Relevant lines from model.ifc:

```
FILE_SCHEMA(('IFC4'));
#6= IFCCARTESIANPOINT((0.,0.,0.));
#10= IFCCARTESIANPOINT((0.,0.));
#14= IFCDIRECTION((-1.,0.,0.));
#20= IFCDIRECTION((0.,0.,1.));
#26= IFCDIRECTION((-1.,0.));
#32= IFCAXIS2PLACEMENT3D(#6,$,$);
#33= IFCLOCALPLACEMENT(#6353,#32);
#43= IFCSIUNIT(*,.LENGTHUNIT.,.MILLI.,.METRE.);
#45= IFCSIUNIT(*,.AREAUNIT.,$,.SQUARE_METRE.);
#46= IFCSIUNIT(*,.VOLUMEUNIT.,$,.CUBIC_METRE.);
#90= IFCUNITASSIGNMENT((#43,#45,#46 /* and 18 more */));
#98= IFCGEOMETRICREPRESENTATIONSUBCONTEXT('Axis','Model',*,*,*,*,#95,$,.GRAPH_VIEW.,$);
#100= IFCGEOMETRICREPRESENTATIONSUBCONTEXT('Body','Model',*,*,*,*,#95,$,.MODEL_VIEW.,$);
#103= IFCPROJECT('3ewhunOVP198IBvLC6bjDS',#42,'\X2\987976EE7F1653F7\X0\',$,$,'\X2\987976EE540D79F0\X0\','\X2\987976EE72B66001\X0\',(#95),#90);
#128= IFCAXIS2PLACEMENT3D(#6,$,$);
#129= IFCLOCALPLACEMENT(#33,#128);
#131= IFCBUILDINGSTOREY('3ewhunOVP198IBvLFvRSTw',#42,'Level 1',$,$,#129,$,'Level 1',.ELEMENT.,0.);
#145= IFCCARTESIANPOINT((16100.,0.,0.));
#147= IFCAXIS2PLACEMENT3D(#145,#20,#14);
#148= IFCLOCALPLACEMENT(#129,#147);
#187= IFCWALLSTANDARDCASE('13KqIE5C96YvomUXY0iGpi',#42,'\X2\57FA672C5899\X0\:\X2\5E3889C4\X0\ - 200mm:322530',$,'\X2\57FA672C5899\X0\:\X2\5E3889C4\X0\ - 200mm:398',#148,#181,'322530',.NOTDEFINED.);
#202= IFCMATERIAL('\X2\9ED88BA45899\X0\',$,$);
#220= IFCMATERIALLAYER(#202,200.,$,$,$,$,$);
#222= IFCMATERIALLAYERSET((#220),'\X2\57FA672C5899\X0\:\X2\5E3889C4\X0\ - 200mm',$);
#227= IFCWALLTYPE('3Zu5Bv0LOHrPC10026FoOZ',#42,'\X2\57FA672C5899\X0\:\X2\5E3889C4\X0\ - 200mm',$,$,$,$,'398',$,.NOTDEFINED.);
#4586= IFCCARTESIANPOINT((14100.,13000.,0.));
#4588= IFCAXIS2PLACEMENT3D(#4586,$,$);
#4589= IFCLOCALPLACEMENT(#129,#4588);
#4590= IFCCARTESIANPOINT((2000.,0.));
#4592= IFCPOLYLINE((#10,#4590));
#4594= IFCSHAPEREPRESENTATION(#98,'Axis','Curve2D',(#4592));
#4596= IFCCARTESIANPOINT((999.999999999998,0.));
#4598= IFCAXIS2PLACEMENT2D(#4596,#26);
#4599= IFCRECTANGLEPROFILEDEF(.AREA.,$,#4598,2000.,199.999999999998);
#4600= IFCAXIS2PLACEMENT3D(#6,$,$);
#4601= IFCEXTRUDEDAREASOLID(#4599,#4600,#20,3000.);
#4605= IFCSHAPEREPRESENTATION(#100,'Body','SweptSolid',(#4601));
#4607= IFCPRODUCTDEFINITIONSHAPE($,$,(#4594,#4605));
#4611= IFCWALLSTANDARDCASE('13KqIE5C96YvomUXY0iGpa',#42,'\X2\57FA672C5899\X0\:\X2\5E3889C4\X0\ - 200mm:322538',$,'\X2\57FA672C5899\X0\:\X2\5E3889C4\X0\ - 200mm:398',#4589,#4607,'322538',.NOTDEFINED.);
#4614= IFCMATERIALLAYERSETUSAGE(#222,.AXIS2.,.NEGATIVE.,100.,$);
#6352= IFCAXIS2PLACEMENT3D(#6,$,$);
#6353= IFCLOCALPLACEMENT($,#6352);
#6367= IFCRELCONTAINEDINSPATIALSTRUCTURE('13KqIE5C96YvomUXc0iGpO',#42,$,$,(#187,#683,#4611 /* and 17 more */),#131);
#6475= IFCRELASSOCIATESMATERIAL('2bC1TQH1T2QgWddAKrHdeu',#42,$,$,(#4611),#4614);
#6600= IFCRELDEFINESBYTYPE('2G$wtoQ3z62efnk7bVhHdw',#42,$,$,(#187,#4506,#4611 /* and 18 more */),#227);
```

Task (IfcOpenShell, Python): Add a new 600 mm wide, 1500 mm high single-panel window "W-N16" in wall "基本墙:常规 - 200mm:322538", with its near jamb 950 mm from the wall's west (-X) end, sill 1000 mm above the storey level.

```python
import numpy as np
import ifcopenshell
import ifcopenshell.api.feature
import ifcopenshell.api.geometry
import ifcopenshell.api.root
import ifcopenshell.api.spatial
import ifcopenshell.geom
import ifcopenshell.util.element
import ifcopenshell.util.placement
import ifcopenshell.util.representation
import ifcopenshell.util.shape
import ifcopenshell.util.unit

model = ifcopenshell.open("model.ifc")
unit_scale = ifcopenshell.util.unit.calculate_unit_scale(model)
settings = ifcopenshell.geom.settings()


def volume(element):
    """Net volume in cubic metres, openings subtracted."""
    shape = ifcopenshell.geom.create_shape(settings, element)
    return ifcopenshell.util.shape.get_volume(shape.geometry)


wall = model.by_guid("13KqIE5C96YvomUXY0iGpa")
storey = ifcopenshell.util.element.get_container(wall, ifc_class="IfcBuildingStorey")
context = ifcopenshell.util.representation.get_context(model, "Model", "Body", "MODEL_VIEW")
before = volume(wall)

width, height, from_end, sill = 0.6, 1.5, 0.95, 1  # metres

# The wall runs along its own X axis, and the end named is its -X end.
wall_shape = ifcopenshell.geom.create_shape(settings, wall)
x, y, z = ifcopenshell.util.shape.get_vertices(wall_shape.geometry).T
start = x.min() + from_end
face, thickness = float(y.min()), float(y.max() - y.min())
wall_matrix = ifcopenshell.util.placement.get_local_placement(wall.ObjectPlacement)
level = ifcopenshell.util.placement.get_local_placement(storey.ObjectPlacement)[2, 3]


def in_wall(x, y):
    """Placement at x, y metres in the wall's axes, at sill height."""
    matrix = wall_matrix.copy()
    matrix[:, 3] = wall_matrix @ np.array([x / unit_scale, y / unit_scale, 0.0, 1.0])
    matrix[2, 3] = level + sill / unit_scale
    return matrix


# Opening: a box that overshoots both wall faces by 50 mm.
opening = ifcopenshell.api.root.create_entity(model, ifc_class="IfcOpeningElement", predefined_type="OPENING")
box = ifcopenshell.api.geometry.add_wall_representation(
    model, context=context, length=width, height=height, thickness=thickness + 0.1
)
ifcopenshell.api.geometry.assign_representation(model, product=opening, representation=box)
ifcopenshell.api.geometry.edit_object_placement(model, product=opening, matrix=in_wall(start, face - 0.05), is_si=False)
ifcopenshell.api.feature.add_feature(model, feature=opening, element=wall)

window = ifcopenshell.api.root.create_entity(model, ifc_class="IfcWindow", name="W-N16", predefined_type="WINDOW")
window.OverallWidth, window.OverallHeight = width / unit_scale, height / unit_scale
window.PartitioningType = "SINGLE_PANEL"
body = ifcopenshell.api.geometry.add_window_representation(
    model,
    context=context,
    overall_width=window.OverallWidth,
    overall_height=window.OverallHeight,
    partition_type="SINGLE_PANEL",
)
ifcopenshell.api.geometry.assign_representation(model, product=window, representation=body)
ifcopenshell.api.spatial.assign_container(model, products=[window], relating_structure=storey)
ifcopenshell.api.feature.add_filling(model, opening=opening, element=window)

# Centre the window in the wall's thickness.
ifcopenshell.api.geometry.edit_object_placement(model, product=window, matrix=in_wall(start, face), is_si=False)
window_shape = ifcopenshell.geom.create_shape(settings, window)
depth = ifcopenshell.util.shape.get_vertices(window_shape.geometry)[:, 1]
offset = face + thickness / 2 - (depth.min() + depth.max()) / 2
ifcopenshell.api.geometry.edit_object_placement(model, product=window, matrix=in_wall(start, offset), is_si=False)

after = volume(wall)

print(f"wall volume {before:.3f} -> {after:.3f} m3")

model.write("model_edited.ifc")
```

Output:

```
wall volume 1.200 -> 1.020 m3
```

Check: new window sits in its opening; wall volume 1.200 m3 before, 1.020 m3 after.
